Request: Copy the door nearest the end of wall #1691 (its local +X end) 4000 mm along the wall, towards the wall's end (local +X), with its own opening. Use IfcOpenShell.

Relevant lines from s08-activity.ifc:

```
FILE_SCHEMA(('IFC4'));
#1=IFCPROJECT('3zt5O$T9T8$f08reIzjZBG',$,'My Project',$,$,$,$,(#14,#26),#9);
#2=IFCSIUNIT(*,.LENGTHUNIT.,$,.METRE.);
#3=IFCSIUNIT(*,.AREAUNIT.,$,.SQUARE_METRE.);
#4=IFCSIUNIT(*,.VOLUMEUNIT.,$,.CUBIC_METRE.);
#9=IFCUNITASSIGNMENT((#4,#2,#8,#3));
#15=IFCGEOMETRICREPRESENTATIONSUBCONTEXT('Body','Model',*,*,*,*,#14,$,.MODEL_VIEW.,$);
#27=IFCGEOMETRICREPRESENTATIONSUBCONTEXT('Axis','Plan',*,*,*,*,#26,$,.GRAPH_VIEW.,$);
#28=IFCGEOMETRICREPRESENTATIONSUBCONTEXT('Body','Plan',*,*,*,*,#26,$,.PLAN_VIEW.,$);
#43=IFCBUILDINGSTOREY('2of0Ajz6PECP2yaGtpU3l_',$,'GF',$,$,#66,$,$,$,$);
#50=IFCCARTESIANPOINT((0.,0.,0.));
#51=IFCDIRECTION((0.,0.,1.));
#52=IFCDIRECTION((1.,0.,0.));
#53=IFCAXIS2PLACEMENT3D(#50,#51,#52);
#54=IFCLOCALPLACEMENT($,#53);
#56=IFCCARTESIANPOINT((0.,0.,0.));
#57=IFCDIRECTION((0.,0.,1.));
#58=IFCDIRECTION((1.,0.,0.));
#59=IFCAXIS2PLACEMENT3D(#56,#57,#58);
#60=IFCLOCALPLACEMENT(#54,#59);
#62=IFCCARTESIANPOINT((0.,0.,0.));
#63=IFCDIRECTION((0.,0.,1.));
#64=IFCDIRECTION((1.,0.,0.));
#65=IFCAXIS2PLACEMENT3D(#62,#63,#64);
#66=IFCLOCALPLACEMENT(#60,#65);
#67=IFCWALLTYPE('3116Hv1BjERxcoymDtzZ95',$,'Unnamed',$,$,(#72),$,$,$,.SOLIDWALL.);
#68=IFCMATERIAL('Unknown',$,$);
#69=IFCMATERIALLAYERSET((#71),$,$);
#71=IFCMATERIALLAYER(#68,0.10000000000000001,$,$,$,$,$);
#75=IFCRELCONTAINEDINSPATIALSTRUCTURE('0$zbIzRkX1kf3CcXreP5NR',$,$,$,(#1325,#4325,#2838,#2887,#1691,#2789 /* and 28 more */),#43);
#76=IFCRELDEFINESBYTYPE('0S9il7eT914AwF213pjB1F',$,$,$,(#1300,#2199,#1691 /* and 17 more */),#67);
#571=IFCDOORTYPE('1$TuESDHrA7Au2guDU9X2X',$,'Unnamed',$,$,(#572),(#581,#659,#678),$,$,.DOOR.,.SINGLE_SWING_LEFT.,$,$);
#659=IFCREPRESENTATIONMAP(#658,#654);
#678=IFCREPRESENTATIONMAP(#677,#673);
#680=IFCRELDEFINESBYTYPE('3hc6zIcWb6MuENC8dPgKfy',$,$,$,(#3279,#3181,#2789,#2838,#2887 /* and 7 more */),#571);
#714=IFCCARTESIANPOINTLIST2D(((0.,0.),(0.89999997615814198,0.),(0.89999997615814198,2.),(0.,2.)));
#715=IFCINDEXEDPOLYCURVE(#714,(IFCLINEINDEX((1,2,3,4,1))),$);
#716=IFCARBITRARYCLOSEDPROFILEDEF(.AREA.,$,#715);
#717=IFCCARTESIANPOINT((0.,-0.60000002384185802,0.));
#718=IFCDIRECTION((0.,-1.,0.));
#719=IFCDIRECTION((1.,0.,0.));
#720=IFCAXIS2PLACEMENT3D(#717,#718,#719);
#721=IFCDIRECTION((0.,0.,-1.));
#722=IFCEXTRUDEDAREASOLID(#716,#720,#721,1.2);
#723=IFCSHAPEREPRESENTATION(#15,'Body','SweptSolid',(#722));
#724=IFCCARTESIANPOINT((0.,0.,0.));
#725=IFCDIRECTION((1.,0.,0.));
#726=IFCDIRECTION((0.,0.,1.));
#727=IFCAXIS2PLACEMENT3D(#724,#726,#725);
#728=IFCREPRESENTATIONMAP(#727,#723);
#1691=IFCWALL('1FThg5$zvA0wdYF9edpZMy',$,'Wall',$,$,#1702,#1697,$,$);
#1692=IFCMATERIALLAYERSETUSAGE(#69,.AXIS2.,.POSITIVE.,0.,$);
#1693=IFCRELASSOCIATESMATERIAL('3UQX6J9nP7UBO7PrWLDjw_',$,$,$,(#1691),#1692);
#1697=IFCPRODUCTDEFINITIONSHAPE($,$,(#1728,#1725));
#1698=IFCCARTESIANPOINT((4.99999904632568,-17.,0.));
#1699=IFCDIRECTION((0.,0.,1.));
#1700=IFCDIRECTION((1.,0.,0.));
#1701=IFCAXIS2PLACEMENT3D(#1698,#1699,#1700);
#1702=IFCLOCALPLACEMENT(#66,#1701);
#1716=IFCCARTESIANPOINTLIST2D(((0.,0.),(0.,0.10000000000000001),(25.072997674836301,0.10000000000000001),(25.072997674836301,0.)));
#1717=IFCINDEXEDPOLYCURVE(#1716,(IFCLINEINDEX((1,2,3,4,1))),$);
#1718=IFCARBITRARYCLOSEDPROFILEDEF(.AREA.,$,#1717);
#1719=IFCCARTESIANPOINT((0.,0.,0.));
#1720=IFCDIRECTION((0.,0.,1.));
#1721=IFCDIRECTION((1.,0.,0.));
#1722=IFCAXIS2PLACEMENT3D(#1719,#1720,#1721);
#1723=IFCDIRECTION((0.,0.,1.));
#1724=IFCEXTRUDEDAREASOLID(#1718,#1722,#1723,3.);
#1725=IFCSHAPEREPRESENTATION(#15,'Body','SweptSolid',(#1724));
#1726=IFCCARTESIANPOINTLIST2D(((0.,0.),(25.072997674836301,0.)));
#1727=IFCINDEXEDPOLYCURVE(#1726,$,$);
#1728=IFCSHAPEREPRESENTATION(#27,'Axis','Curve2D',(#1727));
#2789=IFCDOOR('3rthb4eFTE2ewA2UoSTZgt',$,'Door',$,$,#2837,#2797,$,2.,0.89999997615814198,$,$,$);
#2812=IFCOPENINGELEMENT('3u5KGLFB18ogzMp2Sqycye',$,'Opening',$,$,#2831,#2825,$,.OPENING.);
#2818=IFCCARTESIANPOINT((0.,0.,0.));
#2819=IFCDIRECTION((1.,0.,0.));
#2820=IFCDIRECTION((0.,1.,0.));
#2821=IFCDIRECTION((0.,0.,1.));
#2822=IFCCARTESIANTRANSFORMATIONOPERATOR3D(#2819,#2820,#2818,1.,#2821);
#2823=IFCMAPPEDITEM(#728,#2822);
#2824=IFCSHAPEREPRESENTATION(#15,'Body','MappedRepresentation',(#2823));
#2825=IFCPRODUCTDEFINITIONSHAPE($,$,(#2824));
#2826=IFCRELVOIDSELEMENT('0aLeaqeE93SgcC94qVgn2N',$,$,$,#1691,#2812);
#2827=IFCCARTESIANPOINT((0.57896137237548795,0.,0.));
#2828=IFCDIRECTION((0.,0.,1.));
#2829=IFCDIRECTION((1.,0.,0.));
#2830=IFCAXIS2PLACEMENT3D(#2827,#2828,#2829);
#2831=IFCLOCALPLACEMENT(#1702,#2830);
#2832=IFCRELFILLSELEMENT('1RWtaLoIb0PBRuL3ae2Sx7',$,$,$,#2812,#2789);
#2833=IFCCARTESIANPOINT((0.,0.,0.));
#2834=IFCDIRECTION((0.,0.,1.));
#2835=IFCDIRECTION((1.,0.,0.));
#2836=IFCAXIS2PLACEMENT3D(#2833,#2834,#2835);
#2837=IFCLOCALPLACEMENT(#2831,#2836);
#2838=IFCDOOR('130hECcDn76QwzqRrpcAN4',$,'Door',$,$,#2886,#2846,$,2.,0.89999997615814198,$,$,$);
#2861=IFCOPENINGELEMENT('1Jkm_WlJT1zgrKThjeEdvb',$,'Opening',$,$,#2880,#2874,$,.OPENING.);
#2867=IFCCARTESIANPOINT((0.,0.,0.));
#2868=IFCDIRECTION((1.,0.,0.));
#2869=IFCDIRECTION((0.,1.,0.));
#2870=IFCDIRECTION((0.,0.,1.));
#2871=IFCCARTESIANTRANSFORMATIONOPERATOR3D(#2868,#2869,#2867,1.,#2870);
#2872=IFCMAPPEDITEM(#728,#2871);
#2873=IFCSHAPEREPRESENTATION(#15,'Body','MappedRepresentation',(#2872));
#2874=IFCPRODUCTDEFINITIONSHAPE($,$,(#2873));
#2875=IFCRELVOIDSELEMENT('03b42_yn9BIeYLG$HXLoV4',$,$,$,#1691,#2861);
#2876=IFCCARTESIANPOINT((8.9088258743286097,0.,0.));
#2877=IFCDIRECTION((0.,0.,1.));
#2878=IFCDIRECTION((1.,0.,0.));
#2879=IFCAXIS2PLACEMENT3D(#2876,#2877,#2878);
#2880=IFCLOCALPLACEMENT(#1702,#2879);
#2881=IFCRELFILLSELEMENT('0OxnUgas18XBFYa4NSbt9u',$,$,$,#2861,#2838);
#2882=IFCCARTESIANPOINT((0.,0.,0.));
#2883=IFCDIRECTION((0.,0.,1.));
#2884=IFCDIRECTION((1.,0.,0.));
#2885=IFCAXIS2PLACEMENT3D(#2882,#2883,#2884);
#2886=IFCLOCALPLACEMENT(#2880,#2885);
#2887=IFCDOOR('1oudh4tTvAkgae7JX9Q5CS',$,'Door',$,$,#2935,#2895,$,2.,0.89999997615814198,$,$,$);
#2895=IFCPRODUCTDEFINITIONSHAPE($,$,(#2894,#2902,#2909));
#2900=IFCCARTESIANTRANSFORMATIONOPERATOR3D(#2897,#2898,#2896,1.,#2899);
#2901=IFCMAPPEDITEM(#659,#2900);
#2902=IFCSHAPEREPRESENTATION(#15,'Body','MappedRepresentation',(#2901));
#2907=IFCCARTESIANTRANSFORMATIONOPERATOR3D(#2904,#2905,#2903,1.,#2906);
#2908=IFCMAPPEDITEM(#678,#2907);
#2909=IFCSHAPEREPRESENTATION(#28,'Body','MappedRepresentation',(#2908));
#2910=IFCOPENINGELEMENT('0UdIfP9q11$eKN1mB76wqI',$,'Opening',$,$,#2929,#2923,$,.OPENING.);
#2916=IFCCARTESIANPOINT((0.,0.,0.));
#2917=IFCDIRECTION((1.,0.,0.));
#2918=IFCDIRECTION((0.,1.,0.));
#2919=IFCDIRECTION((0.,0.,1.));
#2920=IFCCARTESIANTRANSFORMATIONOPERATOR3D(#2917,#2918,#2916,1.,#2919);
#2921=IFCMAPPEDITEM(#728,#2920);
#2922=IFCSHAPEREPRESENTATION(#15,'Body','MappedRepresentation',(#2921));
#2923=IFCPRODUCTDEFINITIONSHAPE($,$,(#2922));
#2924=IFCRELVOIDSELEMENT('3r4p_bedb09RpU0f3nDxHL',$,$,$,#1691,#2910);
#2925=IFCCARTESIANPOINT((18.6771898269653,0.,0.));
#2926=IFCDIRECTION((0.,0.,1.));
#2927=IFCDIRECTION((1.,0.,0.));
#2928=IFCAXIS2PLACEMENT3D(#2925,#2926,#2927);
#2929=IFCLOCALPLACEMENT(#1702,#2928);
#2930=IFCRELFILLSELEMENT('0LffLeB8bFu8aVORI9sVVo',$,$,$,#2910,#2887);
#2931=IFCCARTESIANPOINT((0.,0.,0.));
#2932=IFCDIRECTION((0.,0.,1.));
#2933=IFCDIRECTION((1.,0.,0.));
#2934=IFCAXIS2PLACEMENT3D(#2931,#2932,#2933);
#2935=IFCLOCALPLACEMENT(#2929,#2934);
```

```python
import ifcopenshell
import ifcopenshell.api.feature
import ifcopenshell.api.geometry
import ifcopenshell.api.root
import ifcopenshell.geom
import ifcopenshell.util.element
import ifcopenshell.util.placement
import ifcopenshell.util.shape

model = ifcopenshell.open("s08-activity.ifc")
settings = ifcopenshell.geom.settings()


def volume(element):
    """Net volume in cubic metres, openings subtracted."""
    shape = ifcopenshell.geom.create_shape(settings, element)
    return ifcopenshell.util.shape.get_volume(shape.geometry)


door = model.by_id(2887)
opening = door.FillsVoids[0].RelatingOpeningElement
wall = opening.VoidsElements[0].RelatingBuildingElement
before = volume(wall)
shift = ifcopenshell.util.placement.get_local_placement(wall.ObjectPlacement)[:3, 0] * 4.0

# copy_class copies the void relationship, type, container and properties, but no geometry.
new_opening = ifcopenshell.api.root.copy_class(model, product=opening)
new_opening.Representation = ifcopenshell.util.element.copy_deep(
    model, opening.Representation, exclude=["IfcGeometricRepresentationContext", "IfcRepresentationMap"]
)
new_door = ifcopenshell.api.root.copy_class(model, product=door)
new_door.Representation = ifcopenshell.util.element.copy_deep(
    model, door.Representation, exclude=["IfcGeometricRepresentationContext", "IfcRepresentationMap"]
)
ifcopenshell.api.feature.add_filling(model, opening=new_opening, element=new_door)

for old, new in ((opening, new_opening), (door, new_door)):
    matrix = ifcopenshell.util.placement.get_local_placement(old.ObjectPlacement)
    matrix[:3, 3] += shift
    ifcopenshell.api.geometry.edit_object_placement(model, product=new, matrix=matrix, is_si=False)

after = volume(wall)

print(f"wall volume {before:.3f} -> {after:.3f} m3")

model.write("s08-activity_updated.ifc")
```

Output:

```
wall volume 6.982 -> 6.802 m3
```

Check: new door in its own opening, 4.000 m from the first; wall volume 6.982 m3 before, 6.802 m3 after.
